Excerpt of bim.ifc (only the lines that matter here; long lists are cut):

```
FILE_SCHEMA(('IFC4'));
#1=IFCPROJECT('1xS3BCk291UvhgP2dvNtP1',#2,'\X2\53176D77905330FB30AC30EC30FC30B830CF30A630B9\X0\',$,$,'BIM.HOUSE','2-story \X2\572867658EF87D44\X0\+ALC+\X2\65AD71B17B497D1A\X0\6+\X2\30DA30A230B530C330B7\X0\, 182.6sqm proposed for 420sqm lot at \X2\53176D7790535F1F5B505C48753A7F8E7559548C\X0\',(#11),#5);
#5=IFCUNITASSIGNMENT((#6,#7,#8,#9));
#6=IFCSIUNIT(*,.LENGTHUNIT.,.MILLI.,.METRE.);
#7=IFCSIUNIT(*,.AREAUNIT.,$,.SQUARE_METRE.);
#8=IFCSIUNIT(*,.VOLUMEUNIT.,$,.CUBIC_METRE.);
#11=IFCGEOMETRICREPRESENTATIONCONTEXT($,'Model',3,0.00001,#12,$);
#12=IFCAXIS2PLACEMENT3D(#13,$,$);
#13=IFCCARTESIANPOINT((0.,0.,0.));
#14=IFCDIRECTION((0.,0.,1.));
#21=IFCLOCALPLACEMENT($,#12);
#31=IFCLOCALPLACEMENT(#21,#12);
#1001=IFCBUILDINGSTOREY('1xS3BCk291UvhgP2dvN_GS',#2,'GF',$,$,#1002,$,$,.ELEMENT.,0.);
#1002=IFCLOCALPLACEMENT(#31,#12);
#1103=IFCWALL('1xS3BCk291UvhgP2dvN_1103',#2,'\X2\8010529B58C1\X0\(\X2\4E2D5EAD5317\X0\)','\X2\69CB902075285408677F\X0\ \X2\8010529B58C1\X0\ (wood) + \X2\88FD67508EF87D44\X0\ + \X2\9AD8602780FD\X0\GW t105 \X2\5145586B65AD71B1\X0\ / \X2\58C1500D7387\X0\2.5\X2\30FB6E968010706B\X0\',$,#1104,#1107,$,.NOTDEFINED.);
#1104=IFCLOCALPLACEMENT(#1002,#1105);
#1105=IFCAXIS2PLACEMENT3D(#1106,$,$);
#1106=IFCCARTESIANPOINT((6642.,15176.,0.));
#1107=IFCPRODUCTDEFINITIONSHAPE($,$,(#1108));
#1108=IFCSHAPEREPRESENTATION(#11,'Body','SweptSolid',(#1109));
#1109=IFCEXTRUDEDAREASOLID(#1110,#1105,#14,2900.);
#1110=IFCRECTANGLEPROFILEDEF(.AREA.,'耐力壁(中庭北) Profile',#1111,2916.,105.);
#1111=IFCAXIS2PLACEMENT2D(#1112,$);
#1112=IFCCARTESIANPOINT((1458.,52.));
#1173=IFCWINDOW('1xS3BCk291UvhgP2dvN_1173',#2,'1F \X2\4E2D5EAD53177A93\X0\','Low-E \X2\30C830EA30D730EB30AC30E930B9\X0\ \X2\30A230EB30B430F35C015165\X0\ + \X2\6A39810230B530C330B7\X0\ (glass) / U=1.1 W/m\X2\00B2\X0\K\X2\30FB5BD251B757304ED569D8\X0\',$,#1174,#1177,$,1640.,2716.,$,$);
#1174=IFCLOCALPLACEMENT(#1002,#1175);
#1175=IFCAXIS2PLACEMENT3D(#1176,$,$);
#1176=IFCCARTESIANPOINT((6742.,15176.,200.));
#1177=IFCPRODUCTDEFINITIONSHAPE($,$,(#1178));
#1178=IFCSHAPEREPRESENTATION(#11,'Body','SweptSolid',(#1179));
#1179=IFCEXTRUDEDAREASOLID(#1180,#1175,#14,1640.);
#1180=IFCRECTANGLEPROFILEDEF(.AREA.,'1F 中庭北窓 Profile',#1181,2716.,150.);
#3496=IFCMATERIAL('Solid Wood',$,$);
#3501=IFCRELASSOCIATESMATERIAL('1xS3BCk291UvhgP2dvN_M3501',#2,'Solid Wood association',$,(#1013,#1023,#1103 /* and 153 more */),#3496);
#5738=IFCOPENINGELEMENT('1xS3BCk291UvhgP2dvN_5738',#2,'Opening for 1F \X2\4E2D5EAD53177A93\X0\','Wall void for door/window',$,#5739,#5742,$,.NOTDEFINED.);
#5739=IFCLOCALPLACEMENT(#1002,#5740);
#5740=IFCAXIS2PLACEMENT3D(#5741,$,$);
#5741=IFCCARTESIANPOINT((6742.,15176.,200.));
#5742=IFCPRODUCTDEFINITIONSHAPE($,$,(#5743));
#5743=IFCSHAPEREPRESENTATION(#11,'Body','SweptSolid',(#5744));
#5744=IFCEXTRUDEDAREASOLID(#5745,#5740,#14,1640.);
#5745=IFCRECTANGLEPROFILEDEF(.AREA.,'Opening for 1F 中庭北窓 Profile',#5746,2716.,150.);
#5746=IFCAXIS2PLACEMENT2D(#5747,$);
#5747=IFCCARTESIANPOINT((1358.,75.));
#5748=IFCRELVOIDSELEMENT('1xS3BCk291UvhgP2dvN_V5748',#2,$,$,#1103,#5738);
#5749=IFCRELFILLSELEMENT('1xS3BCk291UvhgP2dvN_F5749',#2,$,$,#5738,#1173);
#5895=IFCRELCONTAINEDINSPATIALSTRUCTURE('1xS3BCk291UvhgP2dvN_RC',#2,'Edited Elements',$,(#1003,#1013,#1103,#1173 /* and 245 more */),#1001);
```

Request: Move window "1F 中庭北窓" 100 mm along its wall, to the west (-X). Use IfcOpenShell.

```python
import ifcopenshell
import ifcopenshell.api.geometry
import ifcopenshell.util.placement
import ifcopenshell.util.unit

model = ifcopenshell.open("bim.ifc")
unit_scale = ifcopenshell.util.unit.calculate_unit_scale(model)

window = model.by_id(1173)
opening = window.FillsVoids[0].RelatingOpeningElement
wall = opening.VoidsElements[0].RelatingBuildingElement

wall_matrix = ifcopenshell.util.placement.get_local_placement(wall.ObjectPlacement)
shift = wall_matrix[:3, 0] * -0.1 / unit_scale
before = ifcopenshell.util.placement.get_local_placement(window.ObjectPlacement)[:3, 3].copy()

# The window is not placed relative to its opening, so move both.
for product in (opening, window):
    matrix = ifcopenshell.util.placement.get_local_placement(product.ObjectPlacement)
    matrix[:3, 3] += shift
    ifcopenshell.api.geometry.edit_object_placement(model, product=product, matrix=matrix, is_si=False)

after = ifcopenshell.util.placement.get_local_placement(window.ObjectPlacement)[:3, 3]
print("window moved by", (after - before).round(3) + 0.0)

model.write("bim-out.ifc")
```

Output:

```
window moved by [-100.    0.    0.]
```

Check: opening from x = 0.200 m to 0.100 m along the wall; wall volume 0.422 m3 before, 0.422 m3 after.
